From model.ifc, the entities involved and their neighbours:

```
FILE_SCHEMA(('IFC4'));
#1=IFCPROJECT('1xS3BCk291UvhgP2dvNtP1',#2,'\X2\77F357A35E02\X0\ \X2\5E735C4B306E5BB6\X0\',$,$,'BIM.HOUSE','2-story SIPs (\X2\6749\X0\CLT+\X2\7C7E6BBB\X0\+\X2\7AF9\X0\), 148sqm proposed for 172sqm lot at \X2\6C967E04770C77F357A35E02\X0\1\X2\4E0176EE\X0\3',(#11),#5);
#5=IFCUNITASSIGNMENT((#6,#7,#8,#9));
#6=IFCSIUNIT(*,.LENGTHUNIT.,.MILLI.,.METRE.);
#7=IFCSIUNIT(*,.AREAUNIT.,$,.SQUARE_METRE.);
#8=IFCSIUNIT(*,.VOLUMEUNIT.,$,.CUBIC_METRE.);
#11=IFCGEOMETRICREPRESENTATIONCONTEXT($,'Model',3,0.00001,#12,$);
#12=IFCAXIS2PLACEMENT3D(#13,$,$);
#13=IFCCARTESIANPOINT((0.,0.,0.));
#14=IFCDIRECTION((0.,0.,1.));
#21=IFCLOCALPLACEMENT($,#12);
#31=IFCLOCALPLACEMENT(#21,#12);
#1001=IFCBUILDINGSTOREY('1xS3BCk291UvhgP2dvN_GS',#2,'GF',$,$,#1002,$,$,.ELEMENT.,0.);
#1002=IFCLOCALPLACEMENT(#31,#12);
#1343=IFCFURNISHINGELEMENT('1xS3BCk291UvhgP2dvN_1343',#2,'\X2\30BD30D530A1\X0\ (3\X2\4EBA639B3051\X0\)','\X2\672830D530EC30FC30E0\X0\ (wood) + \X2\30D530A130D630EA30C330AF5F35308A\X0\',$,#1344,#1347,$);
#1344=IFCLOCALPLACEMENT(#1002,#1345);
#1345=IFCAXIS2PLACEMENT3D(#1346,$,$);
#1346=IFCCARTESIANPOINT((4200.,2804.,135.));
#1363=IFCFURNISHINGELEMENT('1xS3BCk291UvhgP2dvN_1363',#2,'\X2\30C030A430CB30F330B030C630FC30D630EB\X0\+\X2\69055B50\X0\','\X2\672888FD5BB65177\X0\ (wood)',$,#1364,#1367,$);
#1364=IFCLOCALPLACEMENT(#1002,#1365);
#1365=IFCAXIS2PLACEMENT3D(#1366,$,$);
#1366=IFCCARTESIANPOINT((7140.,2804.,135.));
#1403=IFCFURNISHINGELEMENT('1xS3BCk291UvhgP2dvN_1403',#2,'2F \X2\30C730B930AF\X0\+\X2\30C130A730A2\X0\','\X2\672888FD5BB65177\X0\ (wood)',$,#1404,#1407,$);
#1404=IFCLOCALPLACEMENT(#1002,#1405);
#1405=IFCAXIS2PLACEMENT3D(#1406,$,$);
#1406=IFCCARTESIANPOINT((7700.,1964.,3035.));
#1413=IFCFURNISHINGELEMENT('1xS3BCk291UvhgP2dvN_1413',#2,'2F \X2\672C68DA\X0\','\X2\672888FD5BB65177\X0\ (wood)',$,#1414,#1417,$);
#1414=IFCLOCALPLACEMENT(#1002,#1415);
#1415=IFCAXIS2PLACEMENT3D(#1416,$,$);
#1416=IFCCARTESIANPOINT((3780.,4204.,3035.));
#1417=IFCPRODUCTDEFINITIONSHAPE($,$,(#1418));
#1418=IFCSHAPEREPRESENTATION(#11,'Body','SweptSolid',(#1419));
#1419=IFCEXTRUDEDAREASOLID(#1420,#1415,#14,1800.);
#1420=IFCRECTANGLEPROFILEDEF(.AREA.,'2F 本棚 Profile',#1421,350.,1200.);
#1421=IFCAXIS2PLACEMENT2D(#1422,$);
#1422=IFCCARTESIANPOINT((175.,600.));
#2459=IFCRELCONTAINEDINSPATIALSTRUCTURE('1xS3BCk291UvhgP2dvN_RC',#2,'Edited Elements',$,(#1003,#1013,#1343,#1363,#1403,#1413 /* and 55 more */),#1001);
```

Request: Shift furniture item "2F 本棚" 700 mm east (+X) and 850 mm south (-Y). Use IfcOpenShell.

```python
import ifcopenshell
import ifcopenshell.api.geometry
import ifcopenshell.util.placement
import ifcopenshell.util.unit

model = ifcopenshell.open("model.ifc")
unit_scale = ifcopenshell.util.unit.calculate_unit_scale(model)

item = model.by_guid("1xS3BCk291UvhgP2dvN_1413")
matrix = ifcopenshell.util.placement.get_local_placement(item.ObjectPlacement)
matrix[0, 3] += 0.7 / unit_scale
matrix[1, 3] -= 0.85 / unit_scale
ifcopenshell.api.geometry.edit_object_placement(model, product=item, matrix=matrix, is_si=False)

print(ifcopenshell.util.placement.get_local_placement(item.ObjectPlacement).round(3) + 0.0)

model.write("model-out.ifc")
```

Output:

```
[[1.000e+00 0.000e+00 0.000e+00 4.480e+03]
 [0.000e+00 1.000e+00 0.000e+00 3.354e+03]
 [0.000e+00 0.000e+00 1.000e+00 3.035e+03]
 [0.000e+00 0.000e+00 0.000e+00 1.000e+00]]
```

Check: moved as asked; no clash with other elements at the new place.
